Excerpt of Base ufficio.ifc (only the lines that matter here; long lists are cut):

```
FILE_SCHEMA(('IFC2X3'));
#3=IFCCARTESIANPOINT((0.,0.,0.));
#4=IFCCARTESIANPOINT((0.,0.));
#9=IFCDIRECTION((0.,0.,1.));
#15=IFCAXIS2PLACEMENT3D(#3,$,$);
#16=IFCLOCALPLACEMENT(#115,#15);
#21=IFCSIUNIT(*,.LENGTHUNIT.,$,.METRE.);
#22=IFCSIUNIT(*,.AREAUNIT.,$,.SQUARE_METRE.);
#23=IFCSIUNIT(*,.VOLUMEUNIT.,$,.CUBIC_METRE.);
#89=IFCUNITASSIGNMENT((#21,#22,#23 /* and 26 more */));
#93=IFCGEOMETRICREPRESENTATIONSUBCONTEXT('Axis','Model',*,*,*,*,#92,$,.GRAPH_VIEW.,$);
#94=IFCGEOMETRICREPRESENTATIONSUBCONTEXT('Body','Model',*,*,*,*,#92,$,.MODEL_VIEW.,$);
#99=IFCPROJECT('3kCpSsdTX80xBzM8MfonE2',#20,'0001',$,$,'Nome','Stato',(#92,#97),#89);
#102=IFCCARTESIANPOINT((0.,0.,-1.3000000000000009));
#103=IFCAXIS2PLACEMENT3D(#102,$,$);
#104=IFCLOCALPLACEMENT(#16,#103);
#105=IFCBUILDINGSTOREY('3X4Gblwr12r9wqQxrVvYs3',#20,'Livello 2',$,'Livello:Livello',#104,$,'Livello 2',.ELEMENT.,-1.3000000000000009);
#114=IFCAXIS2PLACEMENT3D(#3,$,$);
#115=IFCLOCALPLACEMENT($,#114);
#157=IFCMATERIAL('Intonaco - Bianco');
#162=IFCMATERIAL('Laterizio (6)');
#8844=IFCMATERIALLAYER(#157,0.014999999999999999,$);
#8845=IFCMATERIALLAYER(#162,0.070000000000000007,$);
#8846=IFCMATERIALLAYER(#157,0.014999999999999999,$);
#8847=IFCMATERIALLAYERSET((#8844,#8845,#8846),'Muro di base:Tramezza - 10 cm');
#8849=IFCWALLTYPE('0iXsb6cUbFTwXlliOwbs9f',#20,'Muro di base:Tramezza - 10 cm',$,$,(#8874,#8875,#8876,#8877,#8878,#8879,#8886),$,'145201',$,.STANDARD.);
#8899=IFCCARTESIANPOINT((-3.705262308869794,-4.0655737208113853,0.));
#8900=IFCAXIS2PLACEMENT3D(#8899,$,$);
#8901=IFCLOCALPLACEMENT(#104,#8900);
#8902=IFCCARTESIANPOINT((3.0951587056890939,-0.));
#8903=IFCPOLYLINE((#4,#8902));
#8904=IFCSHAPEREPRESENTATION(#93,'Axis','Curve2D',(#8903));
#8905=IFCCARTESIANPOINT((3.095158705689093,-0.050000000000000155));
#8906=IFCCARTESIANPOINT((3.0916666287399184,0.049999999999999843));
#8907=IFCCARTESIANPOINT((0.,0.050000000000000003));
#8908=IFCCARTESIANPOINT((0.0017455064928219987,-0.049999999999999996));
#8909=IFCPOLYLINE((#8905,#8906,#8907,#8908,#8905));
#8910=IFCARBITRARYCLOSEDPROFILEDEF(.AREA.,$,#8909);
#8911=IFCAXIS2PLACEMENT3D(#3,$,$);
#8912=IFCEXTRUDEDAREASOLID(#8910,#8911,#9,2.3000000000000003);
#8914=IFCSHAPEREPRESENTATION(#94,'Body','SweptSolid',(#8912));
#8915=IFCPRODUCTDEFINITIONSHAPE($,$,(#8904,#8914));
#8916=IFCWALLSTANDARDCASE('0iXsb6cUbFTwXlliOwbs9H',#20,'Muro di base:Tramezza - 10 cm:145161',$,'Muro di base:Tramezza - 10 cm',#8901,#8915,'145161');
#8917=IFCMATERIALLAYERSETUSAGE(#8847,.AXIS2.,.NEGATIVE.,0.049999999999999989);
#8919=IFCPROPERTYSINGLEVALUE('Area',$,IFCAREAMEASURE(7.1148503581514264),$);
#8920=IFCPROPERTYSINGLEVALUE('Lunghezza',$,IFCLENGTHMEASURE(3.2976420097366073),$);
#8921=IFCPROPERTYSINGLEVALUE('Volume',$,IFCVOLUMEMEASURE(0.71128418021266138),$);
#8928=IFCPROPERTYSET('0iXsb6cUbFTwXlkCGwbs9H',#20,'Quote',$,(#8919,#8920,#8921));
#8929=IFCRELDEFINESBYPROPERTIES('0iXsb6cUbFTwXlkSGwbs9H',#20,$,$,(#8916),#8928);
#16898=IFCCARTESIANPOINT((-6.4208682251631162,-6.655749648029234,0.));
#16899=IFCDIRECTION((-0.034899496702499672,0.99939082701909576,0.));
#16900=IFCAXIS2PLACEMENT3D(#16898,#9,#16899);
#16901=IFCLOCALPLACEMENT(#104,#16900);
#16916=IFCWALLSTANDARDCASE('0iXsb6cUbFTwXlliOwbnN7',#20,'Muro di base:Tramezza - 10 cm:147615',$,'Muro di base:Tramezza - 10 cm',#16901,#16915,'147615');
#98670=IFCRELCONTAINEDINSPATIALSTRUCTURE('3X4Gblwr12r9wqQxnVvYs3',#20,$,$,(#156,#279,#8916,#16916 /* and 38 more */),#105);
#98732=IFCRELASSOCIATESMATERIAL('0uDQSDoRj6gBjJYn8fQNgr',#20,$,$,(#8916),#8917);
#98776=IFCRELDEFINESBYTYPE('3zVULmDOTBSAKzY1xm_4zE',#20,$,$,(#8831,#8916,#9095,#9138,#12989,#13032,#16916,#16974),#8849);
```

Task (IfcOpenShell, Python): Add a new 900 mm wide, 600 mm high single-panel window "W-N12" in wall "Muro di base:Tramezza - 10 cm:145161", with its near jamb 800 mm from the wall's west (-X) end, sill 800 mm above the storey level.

```python
import numpy as np
import ifcopenshell
import ifcopenshell.api.feature
import ifcopenshell.api.geometry
import ifcopenshell.api.pset
import ifcopenshell.api.root
import ifcopenshell.api.spatial
import ifcopenshell.api.type
import ifcopenshell.geom
import ifcopenshell.util.element
import ifcopenshell.util.placement
import ifcopenshell.util.representation
import ifcopenshell.util.shape
import ifcopenshell.util.unit

model = ifcopenshell.open("Base ufficio.ifc")
unit_scale = ifcopenshell.util.unit.calculate_unit_scale(model)
area_scale = ifcopenshell.util.unit.calculate_unit_scale(model, "AREAUNIT")
volume_scale = ifcopenshell.util.unit.calculate_unit_scale(model, "VOLUMEUNIT")
settings = ifcopenshell.geom.settings()


def volume(element):
    """Net volume in cubic metres, openings subtracted."""
    shape = ifcopenshell.geom.create_shape(settings, element)
    return ifcopenshell.util.shape.get_volume(shape.geometry)


wall = model.by_guid("0iXsb6cUbFTwXlliOwbs9H")
storey = ifcopenshell.util.element.get_container(wall, ifc_class="IfcBuildingStorey")
context = ifcopenshell.util.representation.get_context(model, "Model", "Body", "MODEL_VIEW")
before = volume(wall)

width, height, from_end, sill = 0.9, 0.6, 0.8, 0.8  # metres

# The wall runs along its own X axis, and the end named is its -X end.
wall_shape = ifcopenshell.geom.create_shape(settings, wall)
x, y, z = ifcopenshell.util.shape.get_vertices(wall_shape.geometry).T
start = x.min() + from_end
face, thickness = float(y.min()), float(y.max() - y.min())
wall_matrix = ifcopenshell.util.placement.get_local_placement(wall.ObjectPlacement)
level = ifcopenshell.util.placement.get_local_placement(storey.ObjectPlacement)[2, 3]


def in_wall(x, y):
    """Placement at x, y metres in the wall's axes, at sill height."""
    matrix = wall_matrix.copy()
    matrix[:, 3] = wall_matrix @ np.array([x / unit_scale, y / unit_scale, 0.0, 1.0])
    matrix[2, 3] = level + sill / unit_scale
    return matrix


# Opening: a box that overshoots both wall faces by 50 mm.
opening = ifcopenshell.api.root.create_entity(model, ifc_class="IfcOpeningElement")
box = ifcopenshell.api.geometry.add_wall_representation(
    model, context=context, length=width, height=height, thickness=thickness + 0.1
)
ifcopenshell.api.geometry.assign_representation(model, product=opening, representation=box)
ifcopenshell.api.geometry.edit_object_placement(model, product=opening, matrix=in_wall(start, face - 0.05), is_si=False)
ifcopenshell.api.feature.add_feature(model, feature=opening, element=wall)

window = ifcopenshell.api.root.create_entity(model, ifc_class="IfcWindow", name="W-N12")
window.OverallWidth, window.OverallHeight = width / unit_scale, height / unit_scale
body = ifcopenshell.api.geometry.add_window_representation(
    model,
    context=context,
    overall_width=window.OverallWidth,
    overall_height=window.OverallHeight,
    partition_type="SINGLE_PANEL",
)
ifcopenshell.api.geometry.assign_representation(model, product=window, representation=body)
ifcopenshell.api.spatial.assign_container(model, products=[window], relating_structure=storey)
fills = ifcopenshell.api.feature.add_filling(model, opening=opening, element=window)
fills.OwnerHistory = window.OwnerHistory  # required in IFC2X3

# IFC2X3 keeps the operation on the window style.
style = ifcopenshell.api.root.create_entity(model, ifc_class="IfcWindowStyle", name="W-N12")
style.OperationType, style.ConstructionType = "SINGLE_PANEL", "NOTDEFINED"
style.ParameterTakesPrecedence = style.Sizeable = False
ifcopenshell.api.type.assign_type(model, related_objects=[window], relating_type=style)

# Centre the window in the wall's thickness.
ifcopenshell.api.geometry.edit_object_placement(model, product=window, matrix=in_wall(start, face), is_si=False)
window_shape = ifcopenshell.geom.create_shape(settings, window)
depth = ifcopenshell.util.shape.get_vertices(window_shape.geometry)[:, 1]
offset = face + thickness / 2 - (depth.min() + depth.max()) / 2
ifcopenshell.api.geometry.edit_object_placement(model, product=window, matrix=in_wall(start, offset), is_si=False)

after = volume(wall)

# Update the wall's stored quantities.
pset = model.by_id(ifcopenshell.util.element.get_pset(wall, "Quote", should_inherit=False)["id"])
ifcopenshell.api.pset.edit_pset(model, pset=pset, properties={
    "Area": model.create_entity("IfcAreaMeasure", after / thickness / area_scale),
    "Volume": model.create_entity("IfcVolumeMeasure", after / volume_scale),
})

print(f"wall volume {before:.3f} -> {after:.3f} m3")

model.write("Base ufficio_v2.ifc")
```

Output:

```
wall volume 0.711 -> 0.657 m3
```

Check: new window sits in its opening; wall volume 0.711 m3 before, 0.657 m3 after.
